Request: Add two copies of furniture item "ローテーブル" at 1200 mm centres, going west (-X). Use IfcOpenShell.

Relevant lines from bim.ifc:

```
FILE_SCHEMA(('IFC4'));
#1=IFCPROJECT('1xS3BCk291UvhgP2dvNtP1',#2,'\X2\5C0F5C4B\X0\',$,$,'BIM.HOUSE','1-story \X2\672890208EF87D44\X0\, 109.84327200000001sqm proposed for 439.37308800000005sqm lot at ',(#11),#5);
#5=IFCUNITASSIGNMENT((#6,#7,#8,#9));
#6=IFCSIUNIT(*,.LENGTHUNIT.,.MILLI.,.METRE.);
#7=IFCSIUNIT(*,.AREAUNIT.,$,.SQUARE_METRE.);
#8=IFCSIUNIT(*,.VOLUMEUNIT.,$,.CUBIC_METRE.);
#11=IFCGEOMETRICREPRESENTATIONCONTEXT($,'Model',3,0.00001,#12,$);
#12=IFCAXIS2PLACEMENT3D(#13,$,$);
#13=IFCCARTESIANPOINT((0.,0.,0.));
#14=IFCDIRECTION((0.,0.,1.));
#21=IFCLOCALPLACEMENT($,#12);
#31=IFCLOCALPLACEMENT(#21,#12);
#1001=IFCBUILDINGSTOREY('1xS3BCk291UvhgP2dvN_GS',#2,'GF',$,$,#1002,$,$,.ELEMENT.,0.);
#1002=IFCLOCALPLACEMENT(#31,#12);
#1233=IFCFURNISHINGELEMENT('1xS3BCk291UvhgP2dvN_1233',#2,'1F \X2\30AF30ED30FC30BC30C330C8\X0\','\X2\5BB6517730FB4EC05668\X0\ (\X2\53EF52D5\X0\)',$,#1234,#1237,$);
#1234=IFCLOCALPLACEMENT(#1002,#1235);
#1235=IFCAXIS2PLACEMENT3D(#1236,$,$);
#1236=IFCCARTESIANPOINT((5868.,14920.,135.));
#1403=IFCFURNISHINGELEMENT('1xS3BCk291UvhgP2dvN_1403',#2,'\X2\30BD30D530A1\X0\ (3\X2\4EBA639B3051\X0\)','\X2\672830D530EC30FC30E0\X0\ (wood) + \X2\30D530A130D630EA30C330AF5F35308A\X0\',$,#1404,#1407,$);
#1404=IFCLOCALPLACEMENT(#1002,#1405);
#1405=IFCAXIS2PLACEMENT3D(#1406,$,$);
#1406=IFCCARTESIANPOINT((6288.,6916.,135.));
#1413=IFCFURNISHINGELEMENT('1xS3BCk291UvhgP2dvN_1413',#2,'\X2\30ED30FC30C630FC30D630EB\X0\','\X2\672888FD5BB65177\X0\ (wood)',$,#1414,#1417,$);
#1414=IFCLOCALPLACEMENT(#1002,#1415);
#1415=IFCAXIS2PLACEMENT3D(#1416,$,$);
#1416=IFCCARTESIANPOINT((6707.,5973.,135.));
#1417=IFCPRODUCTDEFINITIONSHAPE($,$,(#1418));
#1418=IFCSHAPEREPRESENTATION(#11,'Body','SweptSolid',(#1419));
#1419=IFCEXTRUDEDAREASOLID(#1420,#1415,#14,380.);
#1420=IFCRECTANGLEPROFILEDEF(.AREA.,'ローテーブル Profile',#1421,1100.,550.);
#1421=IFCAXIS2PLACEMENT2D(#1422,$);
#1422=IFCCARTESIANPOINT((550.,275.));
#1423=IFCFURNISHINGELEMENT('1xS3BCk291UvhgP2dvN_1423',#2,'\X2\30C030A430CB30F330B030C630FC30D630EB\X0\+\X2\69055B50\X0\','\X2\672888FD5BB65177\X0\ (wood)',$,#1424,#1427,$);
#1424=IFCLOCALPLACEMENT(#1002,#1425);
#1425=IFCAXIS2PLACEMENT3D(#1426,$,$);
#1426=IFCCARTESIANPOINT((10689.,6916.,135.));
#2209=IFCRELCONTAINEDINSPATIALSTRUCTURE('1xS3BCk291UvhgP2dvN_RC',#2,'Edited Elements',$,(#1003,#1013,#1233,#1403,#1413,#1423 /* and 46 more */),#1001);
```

```python
import numpy as np
import ifcopenshell
import ifcopenshell.api.geometry
import ifcopenshell.api.root
import ifcopenshell.util.element
import ifcopenshell.util.placement
import ifcopenshell.util.unit

model = ifcopenshell.open("bim.ifc")
unit_scale = ifcopenshell.util.unit.calculate_unit_scale(model)


def reuse_history(source, copy):
    """copy_class also copies each property set's owner history, people and application; keep the originals."""
    for rel in copy.IsDefinedBy:
        if rel.is_a("IfcRelDefinesByProperties") and (history := rel.RelatingPropertyDefinition.OwnerHistory):
            rel.RelatingPropertyDefinition.OwnerHistory = source.OwnerHistory
            ifcopenshell.util.element.remove_deep2(model, history)


source = model.by_guid("1xS3BCk291UvhgP2dvN_1413")
base = ifcopenshell.util.placement.get_local_placement(source.ObjectPlacement)
step = np.array([-1.0, 0.0, 0.0]) * 1.2 / unit_scale

for i in range(1, 3):
    copy = ifcopenshell.api.root.copy_class(model, product=source)
    copy.Representation = ifcopenshell.util.element.copy_deep(
        model, source.Representation, exclude=["IfcGeometricRepresentationContext", "IfcRepresentationMap"]
    )
    reuse_history(source, copy)
    matrix = base.copy()
    matrix[:3, 3] += i * step
    print("added at", matrix[:3, 3].round(3) + 0.0)
    ifcopenshell.api.geometry.edit_object_placement(model, product=copy, matrix=matrix, is_si=False)

model.write("bim-out.ifc")
```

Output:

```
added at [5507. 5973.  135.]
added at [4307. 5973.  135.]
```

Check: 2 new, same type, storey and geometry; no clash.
